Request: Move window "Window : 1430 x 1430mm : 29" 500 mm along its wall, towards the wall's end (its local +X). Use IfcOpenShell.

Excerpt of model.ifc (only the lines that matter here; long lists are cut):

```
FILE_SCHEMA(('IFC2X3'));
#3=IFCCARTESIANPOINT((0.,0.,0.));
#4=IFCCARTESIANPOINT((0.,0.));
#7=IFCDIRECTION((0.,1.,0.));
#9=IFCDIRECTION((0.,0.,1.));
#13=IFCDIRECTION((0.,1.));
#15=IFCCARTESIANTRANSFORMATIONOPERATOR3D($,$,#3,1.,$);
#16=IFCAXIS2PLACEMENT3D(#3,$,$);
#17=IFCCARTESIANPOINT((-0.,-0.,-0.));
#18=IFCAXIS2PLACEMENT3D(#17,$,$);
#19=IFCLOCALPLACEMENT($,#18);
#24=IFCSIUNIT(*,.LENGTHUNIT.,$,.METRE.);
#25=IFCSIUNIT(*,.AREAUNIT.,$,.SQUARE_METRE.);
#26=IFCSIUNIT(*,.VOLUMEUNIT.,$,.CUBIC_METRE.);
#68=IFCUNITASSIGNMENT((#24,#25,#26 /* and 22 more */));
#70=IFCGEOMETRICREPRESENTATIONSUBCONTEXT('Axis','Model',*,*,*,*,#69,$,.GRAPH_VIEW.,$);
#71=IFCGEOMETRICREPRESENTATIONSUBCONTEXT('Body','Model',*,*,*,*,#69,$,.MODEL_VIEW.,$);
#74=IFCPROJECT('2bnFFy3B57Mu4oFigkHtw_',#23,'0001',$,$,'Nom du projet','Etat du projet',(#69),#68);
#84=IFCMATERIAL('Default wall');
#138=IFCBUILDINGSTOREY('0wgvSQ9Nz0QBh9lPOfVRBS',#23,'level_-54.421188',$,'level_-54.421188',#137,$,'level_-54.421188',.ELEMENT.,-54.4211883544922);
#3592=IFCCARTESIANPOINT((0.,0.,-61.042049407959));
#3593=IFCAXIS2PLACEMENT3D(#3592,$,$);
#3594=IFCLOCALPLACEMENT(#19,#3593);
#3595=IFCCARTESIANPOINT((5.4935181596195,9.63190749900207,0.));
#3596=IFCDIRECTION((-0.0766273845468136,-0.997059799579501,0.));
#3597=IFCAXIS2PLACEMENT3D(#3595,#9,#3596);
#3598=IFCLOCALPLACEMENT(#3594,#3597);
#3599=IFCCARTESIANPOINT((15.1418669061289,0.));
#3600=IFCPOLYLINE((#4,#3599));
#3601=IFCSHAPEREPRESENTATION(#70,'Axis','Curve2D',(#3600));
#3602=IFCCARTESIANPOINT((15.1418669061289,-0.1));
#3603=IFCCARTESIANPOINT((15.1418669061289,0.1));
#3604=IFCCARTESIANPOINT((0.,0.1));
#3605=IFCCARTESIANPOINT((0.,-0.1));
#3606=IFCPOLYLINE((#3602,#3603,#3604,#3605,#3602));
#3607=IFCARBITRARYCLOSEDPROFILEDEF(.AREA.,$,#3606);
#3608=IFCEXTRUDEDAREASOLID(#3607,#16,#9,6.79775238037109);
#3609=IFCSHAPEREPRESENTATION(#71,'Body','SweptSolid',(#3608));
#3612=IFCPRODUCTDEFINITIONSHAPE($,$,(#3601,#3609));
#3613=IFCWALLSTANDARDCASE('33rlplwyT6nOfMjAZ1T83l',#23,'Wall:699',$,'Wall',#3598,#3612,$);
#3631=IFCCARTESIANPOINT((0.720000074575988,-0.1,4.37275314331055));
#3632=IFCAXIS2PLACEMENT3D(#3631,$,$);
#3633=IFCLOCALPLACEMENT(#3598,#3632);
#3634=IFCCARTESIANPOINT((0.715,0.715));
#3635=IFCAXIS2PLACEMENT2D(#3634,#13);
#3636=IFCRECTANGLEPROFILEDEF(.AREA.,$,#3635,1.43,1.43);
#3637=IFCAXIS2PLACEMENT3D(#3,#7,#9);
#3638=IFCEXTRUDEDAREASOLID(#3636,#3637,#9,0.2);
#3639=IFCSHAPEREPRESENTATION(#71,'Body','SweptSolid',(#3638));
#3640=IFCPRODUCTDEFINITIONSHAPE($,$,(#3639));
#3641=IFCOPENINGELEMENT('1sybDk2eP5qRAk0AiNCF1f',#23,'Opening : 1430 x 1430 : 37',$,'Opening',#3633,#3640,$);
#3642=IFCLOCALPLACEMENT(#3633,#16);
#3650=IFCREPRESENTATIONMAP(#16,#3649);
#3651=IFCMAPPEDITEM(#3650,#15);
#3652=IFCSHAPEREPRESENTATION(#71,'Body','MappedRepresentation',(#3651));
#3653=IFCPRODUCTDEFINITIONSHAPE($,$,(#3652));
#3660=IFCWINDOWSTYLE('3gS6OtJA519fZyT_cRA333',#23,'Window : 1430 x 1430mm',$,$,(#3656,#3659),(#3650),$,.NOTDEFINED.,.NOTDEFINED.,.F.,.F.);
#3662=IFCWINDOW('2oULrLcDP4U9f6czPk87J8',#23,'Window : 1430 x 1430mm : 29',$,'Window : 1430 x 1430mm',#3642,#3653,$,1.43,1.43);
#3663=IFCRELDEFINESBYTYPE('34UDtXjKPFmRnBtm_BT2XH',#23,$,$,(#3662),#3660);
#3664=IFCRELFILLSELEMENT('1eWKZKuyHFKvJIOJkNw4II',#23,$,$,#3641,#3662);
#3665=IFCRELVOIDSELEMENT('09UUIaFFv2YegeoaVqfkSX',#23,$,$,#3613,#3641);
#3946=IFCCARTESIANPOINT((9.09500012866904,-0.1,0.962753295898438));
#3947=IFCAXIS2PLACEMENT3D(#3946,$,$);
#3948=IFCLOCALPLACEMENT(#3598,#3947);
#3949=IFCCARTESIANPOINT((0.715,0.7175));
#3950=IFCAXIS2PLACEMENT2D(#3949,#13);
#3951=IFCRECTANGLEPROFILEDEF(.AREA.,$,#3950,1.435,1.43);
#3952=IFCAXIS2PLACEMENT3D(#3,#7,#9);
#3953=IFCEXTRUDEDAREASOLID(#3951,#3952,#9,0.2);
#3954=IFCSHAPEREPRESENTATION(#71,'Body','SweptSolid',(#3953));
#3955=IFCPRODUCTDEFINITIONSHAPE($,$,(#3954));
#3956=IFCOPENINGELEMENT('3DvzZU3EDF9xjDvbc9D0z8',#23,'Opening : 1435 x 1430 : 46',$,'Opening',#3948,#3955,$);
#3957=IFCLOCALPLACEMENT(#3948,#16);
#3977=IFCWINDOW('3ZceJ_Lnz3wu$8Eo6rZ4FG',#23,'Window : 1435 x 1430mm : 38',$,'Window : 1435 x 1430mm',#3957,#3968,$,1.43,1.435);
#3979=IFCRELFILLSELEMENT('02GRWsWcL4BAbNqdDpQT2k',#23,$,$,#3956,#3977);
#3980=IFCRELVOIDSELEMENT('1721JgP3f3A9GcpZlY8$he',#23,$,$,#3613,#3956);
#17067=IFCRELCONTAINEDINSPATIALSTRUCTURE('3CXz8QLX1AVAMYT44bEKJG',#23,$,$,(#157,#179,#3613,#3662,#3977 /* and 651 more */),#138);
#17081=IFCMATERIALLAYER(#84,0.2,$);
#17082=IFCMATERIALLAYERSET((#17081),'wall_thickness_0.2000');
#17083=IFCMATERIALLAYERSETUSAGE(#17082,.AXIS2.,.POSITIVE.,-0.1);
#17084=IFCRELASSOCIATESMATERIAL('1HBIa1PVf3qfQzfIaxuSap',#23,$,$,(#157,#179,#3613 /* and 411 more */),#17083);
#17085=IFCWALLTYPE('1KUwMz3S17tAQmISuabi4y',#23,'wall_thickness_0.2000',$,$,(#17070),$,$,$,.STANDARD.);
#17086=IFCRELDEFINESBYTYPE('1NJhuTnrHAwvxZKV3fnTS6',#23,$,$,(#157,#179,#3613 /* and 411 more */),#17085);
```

```python
import ifcopenshell
import ifcopenshell.api.geometry
import ifcopenshell.util.placement

model = ifcopenshell.open("model.ifc")

window = model.by_id(3662)
opening = window.FillsVoids[0].RelatingOpeningElement
wall = opening.VoidsElements[0].RelatingBuildingElement

wall_matrix = ifcopenshell.util.placement.get_local_placement(wall.ObjectPlacement)
shift = wall_matrix[:3, 0] * 0.5
before = ifcopenshell.util.placement.get_local_placement(window.ObjectPlacement)[:3, 3].copy()

# The window is placed relative to its opening, so it follows when the opening moves.
matrix = ifcopenshell.util.placement.get_local_placement(opening.ObjectPlacement)
matrix[:3, 3] += shift
ifcopenshell.api.geometry.edit_object_placement(
    model, product=opening, matrix=matrix, is_si=False, should_transform_children=True
)

after = ifcopenshell.util.placement.get_local_placement(window.ObjectPlacement)[:3, 3]
print("window moved by", (after - before).round(3) + 0.0)

model.write("model_v2.ifc")
```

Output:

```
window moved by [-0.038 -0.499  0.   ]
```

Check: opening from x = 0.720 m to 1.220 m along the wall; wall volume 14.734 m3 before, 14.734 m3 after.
